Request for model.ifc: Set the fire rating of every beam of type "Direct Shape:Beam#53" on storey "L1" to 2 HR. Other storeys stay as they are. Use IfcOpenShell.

First a look at what the model holds.

```python
import ifcopenshell
import ifcopenshell.util.element

model = ifcopenshell.open("model.ifc")
print(model.schema)
storey = next(s for s in model.by_type("IfcBuildingStorey") if s.Name == "L1")
beams = [e for e in ifcopenshell.util.element.get_decomposition(storey) if e.is_a("IfcBeam")]
seen = {}
for e in beams:
    element_type = ifcopenshell.util.element.get_type(e)
    key = (element_type.Name if element_type != e and element_type else None, ifcopenshell.util.element.get_pset(e, "Pset_BeamCommon", "FireRating"))
    seen[key] = seen.get(key, 0) + 1
for (name, value), count in sorted(seen.items(), key=str):
    print(count, "x", name, "|", value)
```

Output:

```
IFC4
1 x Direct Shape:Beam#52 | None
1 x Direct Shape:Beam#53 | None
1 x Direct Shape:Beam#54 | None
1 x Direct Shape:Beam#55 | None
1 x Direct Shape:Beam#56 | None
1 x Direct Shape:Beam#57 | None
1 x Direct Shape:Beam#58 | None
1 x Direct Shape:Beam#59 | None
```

```python
import ifcopenshell
import ifcopenshell.api.pset
import ifcopenshell.util.element

model = ifcopenshell.open("model.ifc")

storey = next(s for s in model.by_type("IfcBuildingStorey") if s.Name == "L1")
beams = [e for e in ifcopenshell.util.element.get_decomposition(storey) if e.is_a("IfcBeam")]

count = 0
for e in beams:
    element_type = ifcopenshell.util.element.get_type(e)
    if element_type in (None, e) or element_type.Name != "Direct Shape:Beam#53":
        continue
    # add_pset returns the element's existing set when there is one.
    pset = ifcopenshell.api.pset.add_pset(model, product=e, name="Pset_BeamCommon")
    ifcopenshell.api.pset.edit_pset(model, pset=pset, properties={"FireRating": "2 HR"})
    count += 1

print(count, "beams updated")

model.write("model_v2.ifc")
```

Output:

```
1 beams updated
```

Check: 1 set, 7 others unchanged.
